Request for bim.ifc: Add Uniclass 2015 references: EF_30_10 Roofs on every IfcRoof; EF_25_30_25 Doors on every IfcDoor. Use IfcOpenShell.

First a look at what the model holds.

```python
import ifcopenshell

model = ifcopenshell.open("bim.ifc")
print(model.schema)
print("classifications:", [c.Name for c in model.by_type("IfcClassification")])
for ifc_class in ("IfcDoor", "IfcRoof", "IfcStair", "IfcWall", "IfcWindow"):
    print(ifc_class, len(model.by_type(ifc_class)))
```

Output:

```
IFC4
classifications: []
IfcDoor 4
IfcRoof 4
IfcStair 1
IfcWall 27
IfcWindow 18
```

```python
import ifcopenshell
import ifcopenshell.api.classification

model = ifcopenshell.open("bim.ifc")

system = ifcopenshell.api.classification.add_classification(model, classification="Uniclass 2015")

codes = {
    "IfcRoof": ("EF_30_10", "Roofs"),
    "IfcDoor": ("EF_25_30_25", "Doors"),
}
for ifc_class, (code, name) in codes.items():
    products = model.by_type(ifc_class)
    ifcopenshell.api.classification.add_reference(
        model, products=products, classification=system, identification=code, name=name
    )
    print(code, len(products))

model.write("bim-out.ifc")
```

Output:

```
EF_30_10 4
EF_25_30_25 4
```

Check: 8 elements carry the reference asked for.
